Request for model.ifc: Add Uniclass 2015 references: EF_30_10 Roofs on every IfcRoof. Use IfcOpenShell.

First a look at what the model holds.

```python
import ifcopenshell

model = ifcopenshell.open("model.ifc")
print(model.schema)
print("classifications:", [c.Name for c in model.by_type("IfcClassification")])
for ifc_class in ("IfcDoor", "IfcRoof", "IfcStair", "IfcWall", "IfcWindow"):
    print(ifc_class, len(model.by_type(ifc_class)))
```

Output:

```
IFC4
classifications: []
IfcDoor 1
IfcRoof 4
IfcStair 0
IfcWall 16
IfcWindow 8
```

```python
import ifcopenshell
import ifcopenshell.api.classification

model = ifcopenshell.open("model.ifc")

system = ifcopenshell.api.classification.add_classification(model, classification="Uniclass 2015")

codes = {
    "IfcRoof": ("EF_30_10", "Roofs"),
}
for ifc_class, (code, name) in codes.items():
    products = model.by_type(ifc_class)
    ifcopenshell.api.classification.add_reference(
        model, products=products, classification=system, identification=code, name=name
    )
    print(code, len(products))

model.write("model_rev.ifc")
```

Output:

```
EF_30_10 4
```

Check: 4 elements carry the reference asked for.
